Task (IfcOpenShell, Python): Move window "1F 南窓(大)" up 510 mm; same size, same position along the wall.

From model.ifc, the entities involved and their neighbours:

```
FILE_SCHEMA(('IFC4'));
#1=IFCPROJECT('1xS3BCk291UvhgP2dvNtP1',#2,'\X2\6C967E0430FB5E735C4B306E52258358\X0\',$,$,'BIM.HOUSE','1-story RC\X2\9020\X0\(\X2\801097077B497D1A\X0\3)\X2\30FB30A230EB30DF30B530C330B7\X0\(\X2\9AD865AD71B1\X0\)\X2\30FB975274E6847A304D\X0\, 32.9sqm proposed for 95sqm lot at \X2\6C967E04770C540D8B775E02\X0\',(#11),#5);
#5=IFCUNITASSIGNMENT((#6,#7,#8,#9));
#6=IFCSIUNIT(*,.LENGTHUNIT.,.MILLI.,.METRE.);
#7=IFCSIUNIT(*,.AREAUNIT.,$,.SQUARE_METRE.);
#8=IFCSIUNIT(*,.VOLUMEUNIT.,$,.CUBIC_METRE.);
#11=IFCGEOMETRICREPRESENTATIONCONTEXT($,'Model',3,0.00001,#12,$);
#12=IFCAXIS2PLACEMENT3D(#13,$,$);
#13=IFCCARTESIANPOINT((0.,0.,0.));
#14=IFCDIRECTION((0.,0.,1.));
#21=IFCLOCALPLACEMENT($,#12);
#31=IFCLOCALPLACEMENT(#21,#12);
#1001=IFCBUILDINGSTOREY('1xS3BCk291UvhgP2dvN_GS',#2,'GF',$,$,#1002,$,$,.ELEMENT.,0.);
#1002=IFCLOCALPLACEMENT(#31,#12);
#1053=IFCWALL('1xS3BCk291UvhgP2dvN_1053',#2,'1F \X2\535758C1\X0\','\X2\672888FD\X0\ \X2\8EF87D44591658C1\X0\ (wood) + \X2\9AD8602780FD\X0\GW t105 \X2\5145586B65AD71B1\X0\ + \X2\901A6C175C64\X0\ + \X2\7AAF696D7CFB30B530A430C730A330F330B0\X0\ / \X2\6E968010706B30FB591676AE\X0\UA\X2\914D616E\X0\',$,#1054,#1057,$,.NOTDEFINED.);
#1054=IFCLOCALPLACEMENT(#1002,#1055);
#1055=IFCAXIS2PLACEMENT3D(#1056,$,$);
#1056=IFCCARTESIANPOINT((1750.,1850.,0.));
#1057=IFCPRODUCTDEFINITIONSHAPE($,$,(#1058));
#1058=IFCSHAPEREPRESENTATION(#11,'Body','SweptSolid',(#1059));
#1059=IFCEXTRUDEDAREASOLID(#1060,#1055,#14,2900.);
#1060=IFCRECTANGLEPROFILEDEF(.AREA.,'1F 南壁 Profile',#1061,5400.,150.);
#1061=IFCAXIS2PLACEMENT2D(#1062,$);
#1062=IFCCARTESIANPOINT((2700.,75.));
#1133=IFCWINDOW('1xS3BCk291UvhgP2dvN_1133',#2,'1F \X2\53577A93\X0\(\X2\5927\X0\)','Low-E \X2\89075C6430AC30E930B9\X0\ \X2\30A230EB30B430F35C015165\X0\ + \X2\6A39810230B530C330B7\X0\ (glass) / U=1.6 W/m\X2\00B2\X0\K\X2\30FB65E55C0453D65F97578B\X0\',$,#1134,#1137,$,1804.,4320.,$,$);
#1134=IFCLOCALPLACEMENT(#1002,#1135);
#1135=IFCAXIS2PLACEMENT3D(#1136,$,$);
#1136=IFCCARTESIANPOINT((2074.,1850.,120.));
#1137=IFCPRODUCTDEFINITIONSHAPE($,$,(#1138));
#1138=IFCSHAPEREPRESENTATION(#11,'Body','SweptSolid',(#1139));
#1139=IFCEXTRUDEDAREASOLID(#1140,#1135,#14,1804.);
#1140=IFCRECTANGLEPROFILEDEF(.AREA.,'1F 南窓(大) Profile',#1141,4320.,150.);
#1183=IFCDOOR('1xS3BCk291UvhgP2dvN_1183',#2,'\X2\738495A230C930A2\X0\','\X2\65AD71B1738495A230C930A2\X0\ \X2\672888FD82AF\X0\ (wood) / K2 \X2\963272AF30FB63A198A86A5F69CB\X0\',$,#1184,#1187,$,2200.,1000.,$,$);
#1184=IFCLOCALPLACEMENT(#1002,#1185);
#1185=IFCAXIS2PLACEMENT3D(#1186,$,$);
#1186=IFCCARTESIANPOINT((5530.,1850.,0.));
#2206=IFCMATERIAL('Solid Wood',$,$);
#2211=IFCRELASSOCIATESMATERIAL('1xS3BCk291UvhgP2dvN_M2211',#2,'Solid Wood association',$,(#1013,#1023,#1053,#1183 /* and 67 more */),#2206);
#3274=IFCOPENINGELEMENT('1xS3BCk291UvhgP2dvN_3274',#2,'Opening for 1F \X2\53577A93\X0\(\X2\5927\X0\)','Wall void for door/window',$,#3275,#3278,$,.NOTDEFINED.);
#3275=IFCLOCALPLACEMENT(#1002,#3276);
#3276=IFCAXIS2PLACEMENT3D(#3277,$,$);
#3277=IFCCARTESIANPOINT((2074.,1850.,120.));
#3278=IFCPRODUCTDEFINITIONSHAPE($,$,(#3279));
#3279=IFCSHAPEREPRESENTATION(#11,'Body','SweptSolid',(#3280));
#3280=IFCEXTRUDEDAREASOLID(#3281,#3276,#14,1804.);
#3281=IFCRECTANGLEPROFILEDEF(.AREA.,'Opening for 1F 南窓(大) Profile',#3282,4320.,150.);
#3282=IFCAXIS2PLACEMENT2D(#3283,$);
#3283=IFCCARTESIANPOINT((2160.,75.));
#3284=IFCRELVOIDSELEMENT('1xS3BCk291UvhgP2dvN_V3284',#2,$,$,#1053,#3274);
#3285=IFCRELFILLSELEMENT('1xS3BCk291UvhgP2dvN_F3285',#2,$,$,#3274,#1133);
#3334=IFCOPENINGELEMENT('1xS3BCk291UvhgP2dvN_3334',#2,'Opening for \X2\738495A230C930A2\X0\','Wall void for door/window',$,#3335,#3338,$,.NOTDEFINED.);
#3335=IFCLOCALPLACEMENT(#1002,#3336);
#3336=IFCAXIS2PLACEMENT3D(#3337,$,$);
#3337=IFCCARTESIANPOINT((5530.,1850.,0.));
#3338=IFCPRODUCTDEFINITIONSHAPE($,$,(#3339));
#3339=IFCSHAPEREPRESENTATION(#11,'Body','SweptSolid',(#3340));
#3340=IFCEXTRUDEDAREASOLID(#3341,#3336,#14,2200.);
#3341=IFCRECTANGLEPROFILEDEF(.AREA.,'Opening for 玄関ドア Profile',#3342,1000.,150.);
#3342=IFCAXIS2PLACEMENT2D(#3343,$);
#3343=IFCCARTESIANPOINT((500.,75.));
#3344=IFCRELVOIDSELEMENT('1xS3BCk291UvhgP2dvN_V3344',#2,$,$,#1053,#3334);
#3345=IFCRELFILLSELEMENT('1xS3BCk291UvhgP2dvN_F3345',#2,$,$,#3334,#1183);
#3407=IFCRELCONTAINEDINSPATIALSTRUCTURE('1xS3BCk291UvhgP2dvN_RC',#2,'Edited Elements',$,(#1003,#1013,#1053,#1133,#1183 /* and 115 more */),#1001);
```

```python
import numpy as np
import ifcopenshell
import ifcopenshell.api.geometry
import ifcopenshell.util.placement
import ifcopenshell.util.unit

model = ifcopenshell.open("model.ifc")
unit_scale = ifcopenshell.util.unit.calculate_unit_scale(model)

window = model.by_guid("1xS3BCk291UvhgP2dvN_1133")
opening = window.FillsVoids[0].RelatingOpeningElement
dz = 0.51 / unit_scale

shift = np.array([0.0, 0.0, dz])
# The window is not placed relative to its opening, so move both.
for product in (opening, window):
    matrix = ifcopenshell.util.placement.get_local_placement(product.ObjectPlacement)
    matrix[:3, 3] += shift
    ifcopenshell.api.geometry.edit_object_placement(model, product=product, matrix=matrix, is_si=False)

print(f"moved by {dz * unit_scale:+.3f} m")

model.write("model_edited.ifc")
```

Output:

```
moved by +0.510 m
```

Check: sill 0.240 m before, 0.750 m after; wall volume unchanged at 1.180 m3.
